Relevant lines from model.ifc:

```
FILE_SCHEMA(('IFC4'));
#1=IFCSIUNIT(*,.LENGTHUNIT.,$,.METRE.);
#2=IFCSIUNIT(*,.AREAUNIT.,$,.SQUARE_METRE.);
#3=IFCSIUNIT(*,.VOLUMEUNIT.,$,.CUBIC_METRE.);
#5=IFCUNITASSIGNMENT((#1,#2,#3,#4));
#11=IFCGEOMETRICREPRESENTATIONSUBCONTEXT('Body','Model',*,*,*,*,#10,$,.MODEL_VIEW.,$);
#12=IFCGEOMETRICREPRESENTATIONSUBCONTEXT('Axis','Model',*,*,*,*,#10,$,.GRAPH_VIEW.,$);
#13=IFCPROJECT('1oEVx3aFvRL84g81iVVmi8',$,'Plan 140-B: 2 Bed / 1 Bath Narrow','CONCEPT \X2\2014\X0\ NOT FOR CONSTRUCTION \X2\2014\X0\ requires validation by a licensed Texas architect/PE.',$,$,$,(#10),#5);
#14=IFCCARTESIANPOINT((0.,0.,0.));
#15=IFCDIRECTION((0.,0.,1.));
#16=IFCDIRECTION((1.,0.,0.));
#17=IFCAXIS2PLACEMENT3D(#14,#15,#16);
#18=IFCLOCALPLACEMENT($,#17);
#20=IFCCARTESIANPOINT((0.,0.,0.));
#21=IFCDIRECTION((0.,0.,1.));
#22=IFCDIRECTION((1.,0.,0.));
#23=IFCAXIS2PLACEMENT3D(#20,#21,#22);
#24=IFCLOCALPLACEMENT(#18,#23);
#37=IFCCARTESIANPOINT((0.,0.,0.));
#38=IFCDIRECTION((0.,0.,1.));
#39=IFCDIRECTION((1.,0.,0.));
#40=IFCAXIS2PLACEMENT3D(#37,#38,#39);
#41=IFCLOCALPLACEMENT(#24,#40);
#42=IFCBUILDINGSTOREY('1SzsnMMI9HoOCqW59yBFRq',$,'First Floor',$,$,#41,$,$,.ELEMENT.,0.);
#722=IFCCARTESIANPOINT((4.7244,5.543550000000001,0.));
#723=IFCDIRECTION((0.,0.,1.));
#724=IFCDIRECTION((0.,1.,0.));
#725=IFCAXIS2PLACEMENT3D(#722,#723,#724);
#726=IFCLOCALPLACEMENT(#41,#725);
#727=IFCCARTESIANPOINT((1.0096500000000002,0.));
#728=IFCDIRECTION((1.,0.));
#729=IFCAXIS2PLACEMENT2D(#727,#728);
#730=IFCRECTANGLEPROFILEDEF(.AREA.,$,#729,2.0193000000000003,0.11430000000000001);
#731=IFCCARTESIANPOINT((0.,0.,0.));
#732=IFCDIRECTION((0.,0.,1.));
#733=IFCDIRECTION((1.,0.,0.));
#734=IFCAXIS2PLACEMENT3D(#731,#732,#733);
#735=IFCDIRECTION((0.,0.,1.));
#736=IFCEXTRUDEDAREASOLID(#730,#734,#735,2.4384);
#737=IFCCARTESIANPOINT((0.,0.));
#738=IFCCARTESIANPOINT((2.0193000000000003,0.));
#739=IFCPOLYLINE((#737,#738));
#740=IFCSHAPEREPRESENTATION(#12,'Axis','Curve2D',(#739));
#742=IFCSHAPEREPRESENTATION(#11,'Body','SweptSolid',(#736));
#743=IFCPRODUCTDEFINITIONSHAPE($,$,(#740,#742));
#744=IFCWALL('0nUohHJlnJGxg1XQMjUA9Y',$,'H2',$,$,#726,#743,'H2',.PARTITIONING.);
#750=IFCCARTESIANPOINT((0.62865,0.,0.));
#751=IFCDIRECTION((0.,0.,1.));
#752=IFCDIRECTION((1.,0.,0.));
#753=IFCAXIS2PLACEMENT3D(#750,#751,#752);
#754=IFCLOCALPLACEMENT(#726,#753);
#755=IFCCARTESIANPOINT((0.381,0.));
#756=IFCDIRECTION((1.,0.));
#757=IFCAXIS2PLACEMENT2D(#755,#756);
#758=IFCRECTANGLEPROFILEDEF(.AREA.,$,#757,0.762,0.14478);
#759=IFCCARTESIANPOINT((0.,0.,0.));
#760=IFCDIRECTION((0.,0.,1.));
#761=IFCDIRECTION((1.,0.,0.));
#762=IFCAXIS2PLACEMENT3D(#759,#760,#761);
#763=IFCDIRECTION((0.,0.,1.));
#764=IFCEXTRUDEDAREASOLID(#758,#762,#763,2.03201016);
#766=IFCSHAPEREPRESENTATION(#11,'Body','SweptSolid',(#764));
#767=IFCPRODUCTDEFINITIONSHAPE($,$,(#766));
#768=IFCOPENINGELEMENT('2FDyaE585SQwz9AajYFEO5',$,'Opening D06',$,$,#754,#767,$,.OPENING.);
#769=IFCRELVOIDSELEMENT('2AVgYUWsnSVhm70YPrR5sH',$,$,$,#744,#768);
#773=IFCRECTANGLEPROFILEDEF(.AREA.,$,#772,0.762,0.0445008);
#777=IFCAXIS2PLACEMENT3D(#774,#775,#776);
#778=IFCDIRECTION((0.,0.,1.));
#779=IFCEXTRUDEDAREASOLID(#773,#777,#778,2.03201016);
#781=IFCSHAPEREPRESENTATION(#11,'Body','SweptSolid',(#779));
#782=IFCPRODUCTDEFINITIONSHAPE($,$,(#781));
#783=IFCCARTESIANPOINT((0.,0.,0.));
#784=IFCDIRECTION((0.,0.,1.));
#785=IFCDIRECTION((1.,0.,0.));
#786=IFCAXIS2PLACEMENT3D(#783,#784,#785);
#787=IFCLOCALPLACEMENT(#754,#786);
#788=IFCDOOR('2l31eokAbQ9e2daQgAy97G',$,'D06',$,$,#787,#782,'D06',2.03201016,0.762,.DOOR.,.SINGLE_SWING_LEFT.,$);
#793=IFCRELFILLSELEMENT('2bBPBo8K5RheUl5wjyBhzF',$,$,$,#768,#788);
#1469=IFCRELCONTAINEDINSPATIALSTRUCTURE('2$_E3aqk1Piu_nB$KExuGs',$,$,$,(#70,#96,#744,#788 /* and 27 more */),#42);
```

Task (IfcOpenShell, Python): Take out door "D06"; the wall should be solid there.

```python
import ifcopenshell
import ifcopenshell.api.feature
import ifcopenshell.api.root
import ifcopenshell.geom
import ifcopenshell.util.shape

model = ifcopenshell.open("model.ifc")
settings = ifcopenshell.geom.settings()


def volume(element):
    """Net volume in cubic metres, openings subtracted."""
    shape = ifcopenshell.geom.create_shape(settings, element)
    return ifcopenshell.util.shape.get_volume(shape.geometry)


door = model.by_id(788)
opening = door.FillsVoids[0].RelatingOpeningElement
wall = opening.VoidsElements[0].RelatingBuildingElement
before = volume(wall)

ifcopenshell.api.root.remove_product(model, product=door)
ifcopenshell.api.feature.remove_feature(model, feature=opening)

after = volume(wall)

print(f"wall volume {before:.3f} -> {after:.3f} m3")

model.write("model_edited.ifc")
```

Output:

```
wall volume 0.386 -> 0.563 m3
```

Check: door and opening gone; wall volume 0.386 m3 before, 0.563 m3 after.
